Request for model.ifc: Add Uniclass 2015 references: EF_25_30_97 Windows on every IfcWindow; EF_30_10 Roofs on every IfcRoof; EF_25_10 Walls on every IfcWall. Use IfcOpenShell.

First a look at what the model holds.

```python
import ifcopenshell

model = ifcopenshell.open("model.ifc")
print(model.schema)
print("classifications:", [c.Name for c in model.by_type("IfcClassification")])
for ifc_class in ("IfcDoor", "IfcRoof", "IfcStair", "IfcWall", "IfcWindow"):
    print(ifc_class, len(model.by_type(ifc_class)))
```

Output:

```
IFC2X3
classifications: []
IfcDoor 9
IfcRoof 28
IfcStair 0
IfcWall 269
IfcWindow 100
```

```python
import ifcopenshell
import ifcopenshell.api.classification

model = ifcopenshell.open("model.ifc")

# IFC2X3 requires Source and Edition and has no link from the project to the system.
system = model.create_entity("IfcClassification", Source="NBS", Edition="2015", Name="Uniclass 2015")

codes = {
    "IfcWindow": ("EF_25_30_97", "Windows"),
    "IfcRoof": ("EF_30_10", "Roofs"),
    "IfcWall": ("EF_25_10", "Walls"),
}
for ifc_class, (code, name) in codes.items():
    products = model.by_type(ifc_class)
    ifcopenshell.api.classification.add_reference(
        model, products=products, classification=system, identification=code, name=name
    )
    print(code, len(products))

model.write("model_updated.ifc")
```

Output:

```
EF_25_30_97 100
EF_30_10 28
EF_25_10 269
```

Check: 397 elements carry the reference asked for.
